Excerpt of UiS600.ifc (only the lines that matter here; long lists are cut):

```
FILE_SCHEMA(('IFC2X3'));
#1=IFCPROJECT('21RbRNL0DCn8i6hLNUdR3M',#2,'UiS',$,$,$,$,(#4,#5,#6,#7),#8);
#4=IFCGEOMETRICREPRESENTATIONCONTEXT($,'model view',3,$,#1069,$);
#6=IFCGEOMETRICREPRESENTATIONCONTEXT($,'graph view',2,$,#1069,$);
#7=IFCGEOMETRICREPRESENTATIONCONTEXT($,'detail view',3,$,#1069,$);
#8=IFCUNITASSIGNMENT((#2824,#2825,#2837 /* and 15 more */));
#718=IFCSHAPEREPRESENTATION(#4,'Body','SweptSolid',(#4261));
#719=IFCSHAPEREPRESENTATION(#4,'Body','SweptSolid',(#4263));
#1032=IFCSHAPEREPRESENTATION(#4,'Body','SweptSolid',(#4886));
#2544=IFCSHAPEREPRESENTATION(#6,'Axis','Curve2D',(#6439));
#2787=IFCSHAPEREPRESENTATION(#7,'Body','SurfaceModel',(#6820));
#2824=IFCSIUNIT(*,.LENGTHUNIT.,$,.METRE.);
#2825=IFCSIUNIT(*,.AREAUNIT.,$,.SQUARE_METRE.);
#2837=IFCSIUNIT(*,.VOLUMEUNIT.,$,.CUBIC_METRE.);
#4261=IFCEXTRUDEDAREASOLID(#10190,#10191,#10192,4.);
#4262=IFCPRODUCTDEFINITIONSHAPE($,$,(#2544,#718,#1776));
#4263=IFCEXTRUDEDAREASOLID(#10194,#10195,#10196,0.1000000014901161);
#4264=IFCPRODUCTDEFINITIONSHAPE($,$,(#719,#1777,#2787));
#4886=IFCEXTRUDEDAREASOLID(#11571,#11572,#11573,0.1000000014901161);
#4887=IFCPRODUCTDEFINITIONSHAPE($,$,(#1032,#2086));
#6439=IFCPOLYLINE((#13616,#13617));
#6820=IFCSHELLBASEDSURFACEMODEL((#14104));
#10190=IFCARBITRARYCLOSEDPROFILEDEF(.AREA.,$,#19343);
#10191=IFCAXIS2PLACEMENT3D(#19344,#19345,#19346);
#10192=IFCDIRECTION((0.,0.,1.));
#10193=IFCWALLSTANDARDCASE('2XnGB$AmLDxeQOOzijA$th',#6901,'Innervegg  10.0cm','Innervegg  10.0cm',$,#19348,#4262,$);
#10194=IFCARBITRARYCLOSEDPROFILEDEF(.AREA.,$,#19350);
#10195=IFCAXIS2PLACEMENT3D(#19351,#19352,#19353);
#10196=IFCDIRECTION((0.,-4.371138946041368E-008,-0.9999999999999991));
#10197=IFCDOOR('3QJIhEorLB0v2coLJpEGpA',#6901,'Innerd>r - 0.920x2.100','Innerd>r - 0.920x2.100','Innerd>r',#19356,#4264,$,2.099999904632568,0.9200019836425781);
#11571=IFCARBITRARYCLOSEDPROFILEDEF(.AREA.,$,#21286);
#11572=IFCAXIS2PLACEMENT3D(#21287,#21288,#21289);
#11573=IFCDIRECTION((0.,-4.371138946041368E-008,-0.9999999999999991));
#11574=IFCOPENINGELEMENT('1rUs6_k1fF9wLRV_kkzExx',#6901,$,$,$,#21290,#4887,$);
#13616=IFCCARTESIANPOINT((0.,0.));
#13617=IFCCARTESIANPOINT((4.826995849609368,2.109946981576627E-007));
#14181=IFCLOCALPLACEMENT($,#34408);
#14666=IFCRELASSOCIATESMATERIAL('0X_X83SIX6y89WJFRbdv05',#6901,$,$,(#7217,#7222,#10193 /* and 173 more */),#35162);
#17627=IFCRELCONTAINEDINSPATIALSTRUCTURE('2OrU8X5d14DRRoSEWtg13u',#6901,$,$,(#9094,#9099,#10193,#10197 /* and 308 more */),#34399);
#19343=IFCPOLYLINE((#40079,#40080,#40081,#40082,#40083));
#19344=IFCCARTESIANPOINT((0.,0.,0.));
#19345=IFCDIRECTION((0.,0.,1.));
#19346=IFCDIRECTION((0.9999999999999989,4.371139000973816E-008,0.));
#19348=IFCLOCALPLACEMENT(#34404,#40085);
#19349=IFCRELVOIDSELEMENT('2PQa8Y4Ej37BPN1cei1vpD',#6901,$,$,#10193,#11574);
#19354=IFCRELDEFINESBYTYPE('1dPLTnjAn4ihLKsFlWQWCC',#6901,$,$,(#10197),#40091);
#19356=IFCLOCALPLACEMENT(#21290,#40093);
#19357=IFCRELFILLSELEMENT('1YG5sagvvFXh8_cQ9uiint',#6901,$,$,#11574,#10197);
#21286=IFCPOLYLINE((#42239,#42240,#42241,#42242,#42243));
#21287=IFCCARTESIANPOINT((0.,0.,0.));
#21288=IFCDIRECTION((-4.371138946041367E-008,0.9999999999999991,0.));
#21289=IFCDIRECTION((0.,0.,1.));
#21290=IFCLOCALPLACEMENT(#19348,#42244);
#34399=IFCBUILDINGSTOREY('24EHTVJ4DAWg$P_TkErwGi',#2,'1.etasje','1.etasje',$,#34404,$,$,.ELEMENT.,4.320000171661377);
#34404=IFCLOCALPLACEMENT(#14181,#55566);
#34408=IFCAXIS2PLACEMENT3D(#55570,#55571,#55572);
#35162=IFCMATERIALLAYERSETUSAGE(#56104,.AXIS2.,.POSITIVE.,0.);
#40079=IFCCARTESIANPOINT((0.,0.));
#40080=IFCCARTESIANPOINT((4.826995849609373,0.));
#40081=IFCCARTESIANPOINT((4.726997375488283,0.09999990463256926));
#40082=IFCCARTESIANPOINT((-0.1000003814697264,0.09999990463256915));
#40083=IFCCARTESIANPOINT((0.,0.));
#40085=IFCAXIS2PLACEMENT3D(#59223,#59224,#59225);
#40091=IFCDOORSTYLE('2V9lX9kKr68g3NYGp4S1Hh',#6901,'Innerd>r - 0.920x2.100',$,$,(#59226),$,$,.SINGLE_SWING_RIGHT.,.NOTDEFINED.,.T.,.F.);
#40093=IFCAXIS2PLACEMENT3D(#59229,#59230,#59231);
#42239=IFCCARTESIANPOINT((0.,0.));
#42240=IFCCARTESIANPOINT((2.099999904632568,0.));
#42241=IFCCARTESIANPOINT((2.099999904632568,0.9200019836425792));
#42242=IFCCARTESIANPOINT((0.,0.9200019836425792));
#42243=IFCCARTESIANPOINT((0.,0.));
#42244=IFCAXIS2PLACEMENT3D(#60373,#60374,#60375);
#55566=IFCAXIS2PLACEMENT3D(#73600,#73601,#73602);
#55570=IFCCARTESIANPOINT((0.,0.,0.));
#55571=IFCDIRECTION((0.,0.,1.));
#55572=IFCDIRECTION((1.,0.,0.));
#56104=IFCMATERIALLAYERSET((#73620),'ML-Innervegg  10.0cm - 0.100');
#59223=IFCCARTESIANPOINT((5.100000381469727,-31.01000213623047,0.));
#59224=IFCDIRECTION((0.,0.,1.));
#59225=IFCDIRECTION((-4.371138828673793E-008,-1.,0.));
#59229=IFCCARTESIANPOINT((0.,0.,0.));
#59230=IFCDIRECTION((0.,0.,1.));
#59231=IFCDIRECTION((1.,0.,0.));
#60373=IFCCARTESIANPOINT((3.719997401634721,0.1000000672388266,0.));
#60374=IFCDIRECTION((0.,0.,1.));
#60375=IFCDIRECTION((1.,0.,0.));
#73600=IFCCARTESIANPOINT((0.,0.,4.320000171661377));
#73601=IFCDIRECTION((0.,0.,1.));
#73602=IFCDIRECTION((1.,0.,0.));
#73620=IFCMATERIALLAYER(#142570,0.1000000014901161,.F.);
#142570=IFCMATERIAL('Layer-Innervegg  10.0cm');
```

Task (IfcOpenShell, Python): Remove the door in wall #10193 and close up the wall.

```python
import ifcopenshell
import ifcopenshell.api.feature
import ifcopenshell.api.root
import ifcopenshell.geom
import ifcopenshell.util.shape

model = ifcopenshell.open("UiS600.ifc")
settings = ifcopenshell.geom.settings()


def volume(element):
    """Net volume in cubic metres, openings subtracted."""
    shape = ifcopenshell.geom.create_shape(settings, element)
    return ifcopenshell.util.shape.get_volume(shape.geometry)


door = model.by_guid("3QJIhEorLB0v2coLJpEGpA")
opening = door.FillsVoids[0].RelatingOpeningElement
wall = opening.VoidsElements[0].RelatingBuildingElement
before = volume(wall)

ifcopenshell.api.root.remove_product(model, product=door)
ifcopenshell.api.feature.remove_feature(model, feature=opening)

after = volume(wall)

print(f"wall volume {before:.3f} -> {after:.3f} m3")

model.write("UiS600_edited.ifc")
```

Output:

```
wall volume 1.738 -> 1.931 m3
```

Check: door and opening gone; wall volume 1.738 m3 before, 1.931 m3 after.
